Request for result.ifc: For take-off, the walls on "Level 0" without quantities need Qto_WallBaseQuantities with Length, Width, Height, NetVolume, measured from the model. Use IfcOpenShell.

First a look at what the model holds.

```python
import ifcopenshell
import ifcopenshell.util.element
import ifcopenshell.util.unit

model = ifcopenshell.open("result.ifc")
print(model.schema)
for unit_type in ("LENGTHUNIT", "AREAUNIT", "VOLUMEUNIT"):
    print(unit_type, ifcopenshell.util.unit.calculate_unit_scale(model, unit_type))
storey = next(s for s in model.by_type("IfcBuildingStorey") if s.Name == "Level 0")
walls = [e for e in ifcopenshell.util.element.get_decomposition(storey) if e.is_a("IfcWall")]
for e in sorted(walls, key=lambda e: e.id()):
    print(e.id(), e.is_a(), e.Name, list(ifcopenshell.util.element.get_psets(e, qtos_only=True)), sep=" | ")
```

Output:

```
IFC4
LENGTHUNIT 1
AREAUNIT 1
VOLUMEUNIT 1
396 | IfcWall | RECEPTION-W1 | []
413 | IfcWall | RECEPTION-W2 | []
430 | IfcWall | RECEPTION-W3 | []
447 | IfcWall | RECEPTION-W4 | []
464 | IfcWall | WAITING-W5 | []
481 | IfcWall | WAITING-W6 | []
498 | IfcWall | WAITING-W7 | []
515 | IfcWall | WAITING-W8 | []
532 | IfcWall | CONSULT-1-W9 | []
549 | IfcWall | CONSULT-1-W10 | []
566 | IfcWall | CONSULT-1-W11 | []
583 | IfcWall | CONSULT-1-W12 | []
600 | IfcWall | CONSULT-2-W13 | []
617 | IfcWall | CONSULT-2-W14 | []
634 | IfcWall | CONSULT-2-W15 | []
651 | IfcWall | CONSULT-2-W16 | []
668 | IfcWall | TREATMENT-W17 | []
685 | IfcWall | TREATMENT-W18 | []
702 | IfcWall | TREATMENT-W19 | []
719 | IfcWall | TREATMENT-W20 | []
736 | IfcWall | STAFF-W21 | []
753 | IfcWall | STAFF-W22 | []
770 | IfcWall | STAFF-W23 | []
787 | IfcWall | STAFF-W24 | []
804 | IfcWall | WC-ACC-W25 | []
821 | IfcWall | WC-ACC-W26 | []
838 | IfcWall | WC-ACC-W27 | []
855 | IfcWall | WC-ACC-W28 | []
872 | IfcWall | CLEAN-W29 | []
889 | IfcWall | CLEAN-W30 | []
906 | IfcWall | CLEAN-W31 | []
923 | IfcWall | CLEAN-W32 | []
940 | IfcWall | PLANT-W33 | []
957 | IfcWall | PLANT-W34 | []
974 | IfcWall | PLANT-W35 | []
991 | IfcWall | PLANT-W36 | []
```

```python
import ifcopenshell
import ifcopenshell.api.pset
import ifcopenshell.geom
import ifcopenshell.util.element
import ifcopenshell.util.shape
import ifcopenshell.util.unit

model = ifcopenshell.open("result.ifc")
unit_scale = ifcopenshell.util.unit.calculate_unit_scale(model)
volume_scale = ifcopenshell.util.unit.calculate_unit_scale(model, "VOLUMEUNIT")
settings = ifcopenshell.geom.settings()

storey = next(s for s in model.by_type("IfcBuildingStorey") if s.Name == "Level 0")
walls = [e for e in ifcopenshell.util.element.get_decomposition(storey) if e.is_a("IfcWall")]

for e in sorted(walls, key=lambda e: e.id()):
    if ifcopenshell.util.element.get_psets(e, qtos_only=True, should_inherit=False):
        continue
    # Geometry comes back in metres, in the element's own axes.
    shape = ifcopenshell.geom.create_shape(settings, e)
    values = {
        "Length": ifcopenshell.util.shape.get_x(shape.geometry) / unit_scale,
        "Width": ifcopenshell.util.shape.get_y(shape.geometry) / unit_scale,
        "Height": ifcopenshell.util.shape.get_z(shape.geometry) / unit_scale,
        "NetVolume": ifcopenshell.util.shape.get_volume(shape.geometry) / volume_scale,
    }
    qto = ifcopenshell.api.pset.add_qto(model, product=e, name="Qto_WallBaseQuantities")
    ifcopenshell.api.pset.edit_qto(model, qto=qto, properties=values)
    print(e.id(), {k: round(v, 3) for k, v in values.items()})

model.write("result_updated.ifc")
```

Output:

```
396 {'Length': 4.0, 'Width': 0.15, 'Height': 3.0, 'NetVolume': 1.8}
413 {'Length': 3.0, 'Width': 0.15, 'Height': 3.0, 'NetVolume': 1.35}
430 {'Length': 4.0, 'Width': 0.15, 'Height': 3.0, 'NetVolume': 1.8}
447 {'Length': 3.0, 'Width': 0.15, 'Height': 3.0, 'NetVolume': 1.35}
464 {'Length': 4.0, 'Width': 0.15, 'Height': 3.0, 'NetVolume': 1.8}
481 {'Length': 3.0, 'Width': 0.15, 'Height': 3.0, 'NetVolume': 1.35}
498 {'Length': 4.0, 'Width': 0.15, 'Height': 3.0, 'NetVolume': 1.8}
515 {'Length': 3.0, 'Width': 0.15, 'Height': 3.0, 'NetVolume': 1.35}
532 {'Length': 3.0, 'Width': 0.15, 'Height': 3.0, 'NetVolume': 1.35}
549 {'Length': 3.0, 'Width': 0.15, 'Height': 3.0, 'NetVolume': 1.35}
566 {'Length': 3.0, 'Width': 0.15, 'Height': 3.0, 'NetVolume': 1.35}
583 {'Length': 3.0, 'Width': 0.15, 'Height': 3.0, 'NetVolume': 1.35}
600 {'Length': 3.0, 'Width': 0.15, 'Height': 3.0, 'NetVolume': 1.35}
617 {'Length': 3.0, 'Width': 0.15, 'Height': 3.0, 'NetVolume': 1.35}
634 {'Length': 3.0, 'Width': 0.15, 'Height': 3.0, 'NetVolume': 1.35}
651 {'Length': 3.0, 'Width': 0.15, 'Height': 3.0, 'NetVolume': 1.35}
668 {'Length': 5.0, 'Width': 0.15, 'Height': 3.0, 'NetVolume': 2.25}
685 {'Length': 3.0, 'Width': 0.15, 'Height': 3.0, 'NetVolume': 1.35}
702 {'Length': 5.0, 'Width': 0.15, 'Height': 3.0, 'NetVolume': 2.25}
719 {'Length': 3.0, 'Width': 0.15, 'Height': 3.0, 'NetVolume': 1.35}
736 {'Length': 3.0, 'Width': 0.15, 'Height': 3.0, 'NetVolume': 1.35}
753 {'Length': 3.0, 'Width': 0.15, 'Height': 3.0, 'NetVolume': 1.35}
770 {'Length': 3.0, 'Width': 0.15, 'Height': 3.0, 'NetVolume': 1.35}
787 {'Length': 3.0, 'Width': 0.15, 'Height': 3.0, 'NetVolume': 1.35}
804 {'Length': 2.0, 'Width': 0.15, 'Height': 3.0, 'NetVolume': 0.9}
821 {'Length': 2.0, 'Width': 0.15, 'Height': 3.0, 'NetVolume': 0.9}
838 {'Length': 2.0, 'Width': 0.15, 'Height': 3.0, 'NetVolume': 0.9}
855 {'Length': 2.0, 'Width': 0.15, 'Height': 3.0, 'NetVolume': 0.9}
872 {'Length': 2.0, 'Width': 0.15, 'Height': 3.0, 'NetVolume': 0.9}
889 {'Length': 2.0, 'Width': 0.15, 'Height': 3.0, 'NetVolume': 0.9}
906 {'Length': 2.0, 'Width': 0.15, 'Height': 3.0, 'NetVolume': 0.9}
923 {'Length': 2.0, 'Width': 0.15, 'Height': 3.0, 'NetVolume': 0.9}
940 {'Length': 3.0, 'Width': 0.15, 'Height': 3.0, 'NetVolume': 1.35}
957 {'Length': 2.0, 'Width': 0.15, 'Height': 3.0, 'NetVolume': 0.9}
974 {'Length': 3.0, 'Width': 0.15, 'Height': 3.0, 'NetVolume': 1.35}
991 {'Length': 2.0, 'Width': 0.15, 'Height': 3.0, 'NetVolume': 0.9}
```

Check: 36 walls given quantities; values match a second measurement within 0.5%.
